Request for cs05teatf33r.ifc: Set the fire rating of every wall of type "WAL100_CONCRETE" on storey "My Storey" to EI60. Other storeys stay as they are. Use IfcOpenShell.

First a look at what the model holds.

```python
import ifcopenshell
import ifcopenshell.util.element

model = ifcopenshell.open("cs05teatf33r.ifc")
print(model.schema)
storey = next(s for s in model.by_type("IfcBuildingStorey") if s.Name == "My Storey")
walls = [e for e in ifcopenshell.util.element.get_decomposition(storey) if e.is_a("IfcWall")]
seen = {}
for e in walls:
    element_type = ifcopenshell.util.element.get_type(e)
    key = (element_type.Name if element_type != e and element_type else None, ifcopenshell.util.element.get_pset(e, "Pset_WallCommon", "FireRating"))
    seen[key] = seen.get(key, 0) + 1
for (name, value), count in sorted(seen.items(), key=str):
    print(count, "x", name, "|", value)
```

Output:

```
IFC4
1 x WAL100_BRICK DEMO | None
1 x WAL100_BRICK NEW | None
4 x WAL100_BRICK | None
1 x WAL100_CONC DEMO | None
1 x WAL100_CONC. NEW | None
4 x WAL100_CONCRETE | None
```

```python
import ifcopenshell
import ifcopenshell.api.pset
import ifcopenshell.util.element

model = ifcopenshell.open("cs05teatf33r.ifc")

storey = next(s for s in model.by_type("IfcBuildingStorey") if s.Name == "My Storey")
walls = [e for e in ifcopenshell.util.element.get_decomposition(storey) if e.is_a("IfcWall")]

count = 0
for e in walls:
    element_type = ifcopenshell.util.element.get_type(e)
    if element_type in (None, e) or element_type.Name != "WAL100_CONCRETE":
        continue
    # add_pset returns the element's existing set when there is one.
    pset = ifcopenshell.api.pset.add_pset(model, product=e, name="Pset_WallCommon")
    ifcopenshell.api.pset.edit_pset(model, pset=pset, properties={"FireRating": "EI60"})
    count += 1

print(count, "walls updated")

model.write("cs05teatf33r_updated.ifc")
```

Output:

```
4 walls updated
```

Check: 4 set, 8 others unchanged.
